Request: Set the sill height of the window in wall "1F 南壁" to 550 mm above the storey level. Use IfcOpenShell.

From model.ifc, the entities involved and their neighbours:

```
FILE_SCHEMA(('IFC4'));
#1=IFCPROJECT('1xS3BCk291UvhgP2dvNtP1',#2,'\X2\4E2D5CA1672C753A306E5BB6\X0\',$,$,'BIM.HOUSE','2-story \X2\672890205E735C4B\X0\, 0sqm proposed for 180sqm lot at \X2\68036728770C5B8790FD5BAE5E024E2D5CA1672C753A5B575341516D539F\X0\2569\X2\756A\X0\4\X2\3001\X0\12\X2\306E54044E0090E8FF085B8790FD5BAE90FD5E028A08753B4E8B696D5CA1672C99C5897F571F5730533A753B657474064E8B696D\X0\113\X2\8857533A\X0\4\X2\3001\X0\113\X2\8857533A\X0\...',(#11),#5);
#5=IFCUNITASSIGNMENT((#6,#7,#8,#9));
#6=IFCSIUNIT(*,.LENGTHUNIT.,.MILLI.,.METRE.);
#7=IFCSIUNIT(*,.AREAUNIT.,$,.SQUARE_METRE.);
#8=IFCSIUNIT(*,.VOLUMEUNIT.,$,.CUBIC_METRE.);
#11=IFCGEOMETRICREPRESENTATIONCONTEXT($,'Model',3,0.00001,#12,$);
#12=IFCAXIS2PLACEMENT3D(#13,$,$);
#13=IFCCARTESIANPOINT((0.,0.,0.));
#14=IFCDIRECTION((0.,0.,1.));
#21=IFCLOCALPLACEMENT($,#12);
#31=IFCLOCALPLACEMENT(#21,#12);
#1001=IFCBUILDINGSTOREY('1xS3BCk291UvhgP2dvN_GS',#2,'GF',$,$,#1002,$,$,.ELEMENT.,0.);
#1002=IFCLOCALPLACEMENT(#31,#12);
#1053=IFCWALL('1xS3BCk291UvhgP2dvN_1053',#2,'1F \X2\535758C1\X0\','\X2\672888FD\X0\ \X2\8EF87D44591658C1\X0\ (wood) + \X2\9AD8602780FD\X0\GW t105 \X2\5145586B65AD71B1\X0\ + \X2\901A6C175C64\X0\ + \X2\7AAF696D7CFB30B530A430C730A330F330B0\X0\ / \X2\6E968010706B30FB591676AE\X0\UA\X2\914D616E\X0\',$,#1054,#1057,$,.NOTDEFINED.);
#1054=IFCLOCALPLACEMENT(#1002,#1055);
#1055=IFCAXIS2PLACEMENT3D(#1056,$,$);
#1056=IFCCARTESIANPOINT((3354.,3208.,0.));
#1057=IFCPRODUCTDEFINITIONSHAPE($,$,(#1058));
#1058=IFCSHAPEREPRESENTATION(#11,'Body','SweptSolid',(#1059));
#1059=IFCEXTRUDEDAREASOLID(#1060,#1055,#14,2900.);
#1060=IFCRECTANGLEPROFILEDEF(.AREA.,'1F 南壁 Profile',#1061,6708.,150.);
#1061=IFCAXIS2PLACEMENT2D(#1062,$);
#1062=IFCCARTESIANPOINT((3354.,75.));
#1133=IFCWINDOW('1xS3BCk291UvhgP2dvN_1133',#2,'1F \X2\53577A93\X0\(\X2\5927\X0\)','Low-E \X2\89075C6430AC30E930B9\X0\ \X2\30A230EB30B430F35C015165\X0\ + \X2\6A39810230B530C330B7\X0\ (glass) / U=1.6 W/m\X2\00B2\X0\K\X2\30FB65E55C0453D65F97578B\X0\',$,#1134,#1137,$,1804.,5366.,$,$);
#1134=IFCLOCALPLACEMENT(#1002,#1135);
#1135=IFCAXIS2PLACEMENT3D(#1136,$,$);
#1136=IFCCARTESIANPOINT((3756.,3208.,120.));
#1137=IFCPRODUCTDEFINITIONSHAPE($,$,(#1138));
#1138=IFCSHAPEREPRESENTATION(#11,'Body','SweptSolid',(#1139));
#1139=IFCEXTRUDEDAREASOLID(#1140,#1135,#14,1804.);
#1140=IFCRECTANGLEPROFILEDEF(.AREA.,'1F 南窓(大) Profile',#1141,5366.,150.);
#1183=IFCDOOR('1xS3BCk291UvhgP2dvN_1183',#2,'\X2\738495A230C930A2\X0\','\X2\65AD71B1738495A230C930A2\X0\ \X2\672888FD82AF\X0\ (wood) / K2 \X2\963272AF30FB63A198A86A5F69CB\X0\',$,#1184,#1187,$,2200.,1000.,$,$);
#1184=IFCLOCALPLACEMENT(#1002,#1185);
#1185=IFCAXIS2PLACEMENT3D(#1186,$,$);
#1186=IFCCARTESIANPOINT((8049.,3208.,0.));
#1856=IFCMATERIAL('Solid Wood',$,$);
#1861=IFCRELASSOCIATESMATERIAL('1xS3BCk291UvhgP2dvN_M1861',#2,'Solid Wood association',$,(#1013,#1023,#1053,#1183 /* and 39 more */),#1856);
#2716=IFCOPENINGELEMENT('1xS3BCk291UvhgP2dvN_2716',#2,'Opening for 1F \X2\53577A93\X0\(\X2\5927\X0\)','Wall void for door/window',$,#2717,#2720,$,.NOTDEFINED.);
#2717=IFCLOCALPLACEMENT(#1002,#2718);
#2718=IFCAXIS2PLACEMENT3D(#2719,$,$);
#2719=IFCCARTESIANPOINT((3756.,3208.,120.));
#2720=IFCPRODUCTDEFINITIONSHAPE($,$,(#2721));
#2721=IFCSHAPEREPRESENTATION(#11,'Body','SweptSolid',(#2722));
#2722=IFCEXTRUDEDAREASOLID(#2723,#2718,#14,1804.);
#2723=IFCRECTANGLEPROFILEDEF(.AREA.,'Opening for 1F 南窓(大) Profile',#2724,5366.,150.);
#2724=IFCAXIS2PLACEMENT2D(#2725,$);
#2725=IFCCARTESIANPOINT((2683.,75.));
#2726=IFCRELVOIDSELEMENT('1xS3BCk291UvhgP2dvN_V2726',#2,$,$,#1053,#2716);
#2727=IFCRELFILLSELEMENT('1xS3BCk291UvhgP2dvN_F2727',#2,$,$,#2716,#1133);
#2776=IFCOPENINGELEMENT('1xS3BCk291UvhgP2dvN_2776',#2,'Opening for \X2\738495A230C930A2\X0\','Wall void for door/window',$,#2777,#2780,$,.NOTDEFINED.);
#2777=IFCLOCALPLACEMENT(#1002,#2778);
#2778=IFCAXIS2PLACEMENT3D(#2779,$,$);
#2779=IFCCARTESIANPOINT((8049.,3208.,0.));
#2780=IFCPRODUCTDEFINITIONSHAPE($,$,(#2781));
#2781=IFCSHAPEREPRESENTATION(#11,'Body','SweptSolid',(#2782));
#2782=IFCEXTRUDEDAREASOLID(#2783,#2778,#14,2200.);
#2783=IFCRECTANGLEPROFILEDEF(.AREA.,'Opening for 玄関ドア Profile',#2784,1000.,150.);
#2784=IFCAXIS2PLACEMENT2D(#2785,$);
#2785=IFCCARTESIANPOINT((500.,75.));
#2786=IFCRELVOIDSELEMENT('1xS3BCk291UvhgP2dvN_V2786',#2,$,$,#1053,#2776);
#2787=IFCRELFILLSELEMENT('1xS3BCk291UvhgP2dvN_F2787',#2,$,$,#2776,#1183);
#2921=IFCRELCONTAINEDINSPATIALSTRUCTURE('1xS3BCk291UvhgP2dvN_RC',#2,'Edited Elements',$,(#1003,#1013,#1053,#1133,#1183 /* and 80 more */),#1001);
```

```python
import numpy as np
import ifcopenshell
import ifcopenshell.api.geometry
import ifcopenshell.geom
import ifcopenshell.util.element
import ifcopenshell.util.placement
import ifcopenshell.util.shape
import ifcopenshell.util.unit

model = ifcopenshell.open("model.ifc")
unit_scale = ifcopenshell.util.unit.calculate_unit_scale(model)

window = model.by_guid("1xS3BCk291UvhgP2dvN_1133")
opening = window.FillsVoids[0].RelatingOpeningElement
storey = ifcopenshell.util.element.get_container(window, ifc_class="IfcBuildingStorey")
level = ifcopenshell.util.placement.get_local_placement(storey.ObjectPlacement)[2, 3]

# The opening's origin need not be at the sill, so measure its lowest point.
shape = ifcopenshell.geom.create_shape(ifcopenshell.geom.settings(), opening)
bottom = ifcopenshell.util.shape.get_shape_bottom_elevation(shape, shape.geometry) / unit_scale
dz = level + 0.55 / unit_scale - bottom

shift = np.array([0.0, 0.0, dz])
# The window is not placed relative to its opening, so move both.
for product in (opening, window):
    matrix = ifcopenshell.util.placement.get_local_placement(product.ObjectPlacement)
    matrix[:3, 3] += shift
    ifcopenshell.api.geometry.edit_object_placement(model, product=product, matrix=matrix, is_si=False)

print(f"moved by {dz * unit_scale:+.3f} m")

model.write("model_rev.ifc")
```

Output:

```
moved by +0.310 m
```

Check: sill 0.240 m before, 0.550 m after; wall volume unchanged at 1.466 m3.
